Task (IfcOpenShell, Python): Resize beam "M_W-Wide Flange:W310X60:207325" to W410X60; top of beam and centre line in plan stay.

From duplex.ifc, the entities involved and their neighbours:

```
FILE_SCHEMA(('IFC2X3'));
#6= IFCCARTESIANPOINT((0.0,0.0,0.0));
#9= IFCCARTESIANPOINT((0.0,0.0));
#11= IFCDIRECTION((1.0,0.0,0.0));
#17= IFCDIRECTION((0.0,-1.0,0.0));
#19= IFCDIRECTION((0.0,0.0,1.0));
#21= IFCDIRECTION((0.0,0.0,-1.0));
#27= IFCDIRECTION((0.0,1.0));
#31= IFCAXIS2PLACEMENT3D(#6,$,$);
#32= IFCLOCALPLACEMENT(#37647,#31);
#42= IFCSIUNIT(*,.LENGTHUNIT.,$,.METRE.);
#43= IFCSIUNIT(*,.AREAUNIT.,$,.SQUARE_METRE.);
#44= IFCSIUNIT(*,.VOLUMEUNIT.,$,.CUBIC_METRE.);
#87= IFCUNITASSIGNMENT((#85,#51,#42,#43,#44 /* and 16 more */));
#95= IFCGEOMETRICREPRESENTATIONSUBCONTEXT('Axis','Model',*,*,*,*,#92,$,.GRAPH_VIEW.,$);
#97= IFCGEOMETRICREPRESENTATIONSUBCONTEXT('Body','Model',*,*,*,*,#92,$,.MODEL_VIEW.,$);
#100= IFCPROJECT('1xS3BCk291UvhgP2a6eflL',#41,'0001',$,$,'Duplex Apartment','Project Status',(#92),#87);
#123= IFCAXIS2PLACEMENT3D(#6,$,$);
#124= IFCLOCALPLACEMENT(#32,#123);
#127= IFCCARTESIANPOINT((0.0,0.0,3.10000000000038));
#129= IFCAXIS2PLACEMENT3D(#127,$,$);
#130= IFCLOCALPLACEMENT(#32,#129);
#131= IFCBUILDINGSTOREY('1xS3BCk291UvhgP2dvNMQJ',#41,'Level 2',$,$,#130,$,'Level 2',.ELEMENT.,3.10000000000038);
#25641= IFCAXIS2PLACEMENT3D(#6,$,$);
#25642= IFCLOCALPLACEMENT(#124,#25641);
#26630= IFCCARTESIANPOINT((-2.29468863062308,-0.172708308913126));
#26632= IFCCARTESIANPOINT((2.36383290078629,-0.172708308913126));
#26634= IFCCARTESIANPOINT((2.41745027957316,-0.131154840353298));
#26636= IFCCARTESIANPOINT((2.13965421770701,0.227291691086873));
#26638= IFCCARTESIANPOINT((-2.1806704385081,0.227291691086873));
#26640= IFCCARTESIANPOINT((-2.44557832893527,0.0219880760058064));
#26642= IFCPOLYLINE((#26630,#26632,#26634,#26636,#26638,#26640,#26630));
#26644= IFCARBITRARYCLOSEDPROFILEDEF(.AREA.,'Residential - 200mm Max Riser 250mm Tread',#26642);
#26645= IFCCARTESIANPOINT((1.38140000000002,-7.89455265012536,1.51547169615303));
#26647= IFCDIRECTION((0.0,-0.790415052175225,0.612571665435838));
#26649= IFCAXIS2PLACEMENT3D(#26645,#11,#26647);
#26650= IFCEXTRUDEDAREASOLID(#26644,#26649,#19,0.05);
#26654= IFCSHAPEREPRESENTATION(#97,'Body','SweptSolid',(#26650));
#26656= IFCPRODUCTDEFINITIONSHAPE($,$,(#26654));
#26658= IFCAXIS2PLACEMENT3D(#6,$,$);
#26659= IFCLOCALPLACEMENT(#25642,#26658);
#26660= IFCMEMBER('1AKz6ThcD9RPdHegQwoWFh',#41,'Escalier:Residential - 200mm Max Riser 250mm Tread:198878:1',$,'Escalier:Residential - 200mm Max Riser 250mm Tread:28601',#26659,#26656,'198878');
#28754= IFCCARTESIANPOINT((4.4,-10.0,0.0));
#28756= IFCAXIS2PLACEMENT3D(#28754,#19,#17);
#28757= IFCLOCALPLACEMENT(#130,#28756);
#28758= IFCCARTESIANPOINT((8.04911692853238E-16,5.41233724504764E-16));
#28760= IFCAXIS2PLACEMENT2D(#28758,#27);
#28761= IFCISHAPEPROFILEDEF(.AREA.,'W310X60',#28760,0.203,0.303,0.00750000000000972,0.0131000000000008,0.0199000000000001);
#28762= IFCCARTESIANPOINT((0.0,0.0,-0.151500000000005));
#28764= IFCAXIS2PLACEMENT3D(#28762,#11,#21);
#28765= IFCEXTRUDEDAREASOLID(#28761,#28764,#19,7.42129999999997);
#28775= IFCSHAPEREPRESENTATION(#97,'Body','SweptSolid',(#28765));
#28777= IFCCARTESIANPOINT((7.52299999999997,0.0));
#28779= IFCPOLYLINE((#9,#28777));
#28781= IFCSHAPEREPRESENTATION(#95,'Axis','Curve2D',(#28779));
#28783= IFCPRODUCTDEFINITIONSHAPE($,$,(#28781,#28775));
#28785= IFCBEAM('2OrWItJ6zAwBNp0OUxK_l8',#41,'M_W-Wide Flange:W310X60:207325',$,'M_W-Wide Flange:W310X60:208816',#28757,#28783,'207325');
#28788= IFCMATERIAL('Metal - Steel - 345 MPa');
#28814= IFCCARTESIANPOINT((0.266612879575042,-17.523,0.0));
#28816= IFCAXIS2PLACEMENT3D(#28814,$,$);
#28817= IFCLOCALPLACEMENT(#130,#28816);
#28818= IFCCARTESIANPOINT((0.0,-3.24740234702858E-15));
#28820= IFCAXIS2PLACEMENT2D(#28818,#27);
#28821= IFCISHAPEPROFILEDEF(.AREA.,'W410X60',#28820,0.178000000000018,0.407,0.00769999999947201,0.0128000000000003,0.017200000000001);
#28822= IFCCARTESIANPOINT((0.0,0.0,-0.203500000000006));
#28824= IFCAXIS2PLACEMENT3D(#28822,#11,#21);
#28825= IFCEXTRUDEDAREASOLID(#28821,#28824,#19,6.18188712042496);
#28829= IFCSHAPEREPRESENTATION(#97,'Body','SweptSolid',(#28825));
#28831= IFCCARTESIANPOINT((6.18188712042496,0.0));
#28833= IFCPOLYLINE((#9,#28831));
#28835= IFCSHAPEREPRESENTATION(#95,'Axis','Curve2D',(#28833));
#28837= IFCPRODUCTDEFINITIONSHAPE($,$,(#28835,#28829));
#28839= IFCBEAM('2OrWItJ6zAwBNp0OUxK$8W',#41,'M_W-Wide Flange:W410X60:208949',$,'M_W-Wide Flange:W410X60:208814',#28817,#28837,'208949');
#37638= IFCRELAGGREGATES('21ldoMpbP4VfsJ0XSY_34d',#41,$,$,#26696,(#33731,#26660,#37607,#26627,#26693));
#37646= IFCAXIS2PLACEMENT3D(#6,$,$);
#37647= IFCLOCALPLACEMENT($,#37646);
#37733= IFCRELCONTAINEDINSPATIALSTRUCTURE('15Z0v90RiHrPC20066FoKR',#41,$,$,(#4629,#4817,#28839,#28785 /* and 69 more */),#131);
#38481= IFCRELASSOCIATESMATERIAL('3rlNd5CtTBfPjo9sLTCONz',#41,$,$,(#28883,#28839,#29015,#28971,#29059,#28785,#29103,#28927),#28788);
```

```python
import ifcopenshell
import ifcopenshell.util.element
import ifcopenshell.util.representation

model = ifcopenshell.open("duplex.ifc")

member = model.by_guid("2OrWItJ6zAwBNp0OUxK_l8")
source = next(p for p in model.by_type("IfcIShapeProfileDef") if p.ProfileName == "W410X60")

body = ifcopenshell.util.representation.get_representation(member, "Model", "Body")
solid = body.Items[0]
old_profile = solid.SweptArea

# Copy the section's sizes but keep this member's own profile position.
profile = ifcopenshell.util.element.copy(model, source)
# Profiles are centred, so shift by half the change in depth to hold the top.
shift = (old_profile.OverallDepth - profile.OverallDepth) / 2
x, y = old_profile.Position.Location.Coordinates
up = (-1.0, 0.0)  # upwards, in the solid's own plane
location = model.createIfcCartesianPoint((x + up[0] * shift, y + up[1] * shift))
profile.Position = model.createIfcAxis2Placement2D(location, old_profile.Position.RefDirection)
solid.SweptArea = profile
if not model.get_total_inverses(old_profile):
    ifcopenshell.util.element.remove_deep2(model, old_profile)
member.Name = member.Name.replace("W310X60", "W410X60")
member.ObjectType = member.ObjectType.replace("W310X60", "W410X60")

print(solid.SweptArea)

model.write("duplex-out.ifc")
```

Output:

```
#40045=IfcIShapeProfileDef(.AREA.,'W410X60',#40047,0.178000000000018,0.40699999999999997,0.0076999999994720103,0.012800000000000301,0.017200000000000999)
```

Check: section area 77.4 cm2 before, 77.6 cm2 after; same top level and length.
